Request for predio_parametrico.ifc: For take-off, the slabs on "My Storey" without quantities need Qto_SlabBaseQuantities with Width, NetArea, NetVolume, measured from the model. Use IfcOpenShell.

First a look at what the model holds.

```python
import ifcopenshell
import ifcopenshell.util.element
import ifcopenshell.util.unit

model = ifcopenshell.open("predio_parametrico.ifc")
print(model.schema)
for unit_type in ("LENGTHUNIT", "AREAUNIT", "VOLUMEUNIT"):
    print(unit_type, ifcopenshell.util.unit.calculate_unit_scale(model, unit_type))
storey = next(s for s in model.by_type("IfcBuildingStorey") if s.Name == "My Storey")
slabs = [e for e in ifcopenshell.util.element.get_decomposition(storey) if e.is_a("IfcSlab")]
for e in sorted(slabs, key=lambda e: e.id()):
    print(e.id(), e.is_a(), e.Name, list(ifcopenshell.util.element.get_psets(e, qtos_only=True)), sep=" | ")
```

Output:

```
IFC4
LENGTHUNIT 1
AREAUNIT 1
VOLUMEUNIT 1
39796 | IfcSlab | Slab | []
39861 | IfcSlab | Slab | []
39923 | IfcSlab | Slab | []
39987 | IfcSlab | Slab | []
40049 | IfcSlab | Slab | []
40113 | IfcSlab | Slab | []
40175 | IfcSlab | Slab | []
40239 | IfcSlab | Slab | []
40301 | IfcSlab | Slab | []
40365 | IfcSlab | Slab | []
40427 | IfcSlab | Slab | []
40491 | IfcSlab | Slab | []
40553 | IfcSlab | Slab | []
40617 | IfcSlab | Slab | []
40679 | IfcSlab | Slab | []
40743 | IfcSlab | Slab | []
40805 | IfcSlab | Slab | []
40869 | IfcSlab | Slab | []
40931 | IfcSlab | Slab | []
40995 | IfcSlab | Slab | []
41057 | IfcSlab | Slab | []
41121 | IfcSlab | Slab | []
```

```python
import ifcopenshell
import ifcopenshell.api.pset
import ifcopenshell.geom
import ifcopenshell.util.element
import ifcopenshell.util.shape
import ifcopenshell.util.unit

model = ifcopenshell.open("predio_parametrico.ifc")
unit_scale = ifcopenshell.util.unit.calculate_unit_scale(model)
area_scale = ifcopenshell.util.unit.calculate_unit_scale(model, "AREAUNIT")
volume_scale = ifcopenshell.util.unit.calculate_unit_scale(model, "VOLUMEUNIT")
settings = ifcopenshell.geom.settings()

storey = next(s for s in model.by_type("IfcBuildingStorey") if s.Name == "My Storey")
slabs = [e for e in ifcopenshell.util.element.get_decomposition(storey) if e.is_a("IfcSlab")]

for e in sorted(slabs, key=lambda e: e.id()):
    if ifcopenshell.util.element.get_psets(e, qtos_only=True, should_inherit=False):
        continue
    # Geometry comes back in metres, in the element's own axes.
    shape = ifcopenshell.geom.create_shape(settings, e)
    values = {
        "Width": ifcopenshell.util.shape.get_z(shape.geometry) / unit_scale,
        "NetArea": ifcopenshell.util.shape.get_footprint_area(shape.geometry) / area_scale,
        "NetVolume": ifcopenshell.util.shape.get_volume(shape.geometry) / volume_scale,
    }
    qto = ifcopenshell.api.pset.add_qto(model, product=e, name="Qto_SlabBaseQuantities")
    ifcopenshell.api.pset.edit_qto(model, qto=qto, properties=values)
    print(e.id(), {k: round(v, 3) for k, v in values.items()})

model.write("predio_parametrico_updated.ifc")
```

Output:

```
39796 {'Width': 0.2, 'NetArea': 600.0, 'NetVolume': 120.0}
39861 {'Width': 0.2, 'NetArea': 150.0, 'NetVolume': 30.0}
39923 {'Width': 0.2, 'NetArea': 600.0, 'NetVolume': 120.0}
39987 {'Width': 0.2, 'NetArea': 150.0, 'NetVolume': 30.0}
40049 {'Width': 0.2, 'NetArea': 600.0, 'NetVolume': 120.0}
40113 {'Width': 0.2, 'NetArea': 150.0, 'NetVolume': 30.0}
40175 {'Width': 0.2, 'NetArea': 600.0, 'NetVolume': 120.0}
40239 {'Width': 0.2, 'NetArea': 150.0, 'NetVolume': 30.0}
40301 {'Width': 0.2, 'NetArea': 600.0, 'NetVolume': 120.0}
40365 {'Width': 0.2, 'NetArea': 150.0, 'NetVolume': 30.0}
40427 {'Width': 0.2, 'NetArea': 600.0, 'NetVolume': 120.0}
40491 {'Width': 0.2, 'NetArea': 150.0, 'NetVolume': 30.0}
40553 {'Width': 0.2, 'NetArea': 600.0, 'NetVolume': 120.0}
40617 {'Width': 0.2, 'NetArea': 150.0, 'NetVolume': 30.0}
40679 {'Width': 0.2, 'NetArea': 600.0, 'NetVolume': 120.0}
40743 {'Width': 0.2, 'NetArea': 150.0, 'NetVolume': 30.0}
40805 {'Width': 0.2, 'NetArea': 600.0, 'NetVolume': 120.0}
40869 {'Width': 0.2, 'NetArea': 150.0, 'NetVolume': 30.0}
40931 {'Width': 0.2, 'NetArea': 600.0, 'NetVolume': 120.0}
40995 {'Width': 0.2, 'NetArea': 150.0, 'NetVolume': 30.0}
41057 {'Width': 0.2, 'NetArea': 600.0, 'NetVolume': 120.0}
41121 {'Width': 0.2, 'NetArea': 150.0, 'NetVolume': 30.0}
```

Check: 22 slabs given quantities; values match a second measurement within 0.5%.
